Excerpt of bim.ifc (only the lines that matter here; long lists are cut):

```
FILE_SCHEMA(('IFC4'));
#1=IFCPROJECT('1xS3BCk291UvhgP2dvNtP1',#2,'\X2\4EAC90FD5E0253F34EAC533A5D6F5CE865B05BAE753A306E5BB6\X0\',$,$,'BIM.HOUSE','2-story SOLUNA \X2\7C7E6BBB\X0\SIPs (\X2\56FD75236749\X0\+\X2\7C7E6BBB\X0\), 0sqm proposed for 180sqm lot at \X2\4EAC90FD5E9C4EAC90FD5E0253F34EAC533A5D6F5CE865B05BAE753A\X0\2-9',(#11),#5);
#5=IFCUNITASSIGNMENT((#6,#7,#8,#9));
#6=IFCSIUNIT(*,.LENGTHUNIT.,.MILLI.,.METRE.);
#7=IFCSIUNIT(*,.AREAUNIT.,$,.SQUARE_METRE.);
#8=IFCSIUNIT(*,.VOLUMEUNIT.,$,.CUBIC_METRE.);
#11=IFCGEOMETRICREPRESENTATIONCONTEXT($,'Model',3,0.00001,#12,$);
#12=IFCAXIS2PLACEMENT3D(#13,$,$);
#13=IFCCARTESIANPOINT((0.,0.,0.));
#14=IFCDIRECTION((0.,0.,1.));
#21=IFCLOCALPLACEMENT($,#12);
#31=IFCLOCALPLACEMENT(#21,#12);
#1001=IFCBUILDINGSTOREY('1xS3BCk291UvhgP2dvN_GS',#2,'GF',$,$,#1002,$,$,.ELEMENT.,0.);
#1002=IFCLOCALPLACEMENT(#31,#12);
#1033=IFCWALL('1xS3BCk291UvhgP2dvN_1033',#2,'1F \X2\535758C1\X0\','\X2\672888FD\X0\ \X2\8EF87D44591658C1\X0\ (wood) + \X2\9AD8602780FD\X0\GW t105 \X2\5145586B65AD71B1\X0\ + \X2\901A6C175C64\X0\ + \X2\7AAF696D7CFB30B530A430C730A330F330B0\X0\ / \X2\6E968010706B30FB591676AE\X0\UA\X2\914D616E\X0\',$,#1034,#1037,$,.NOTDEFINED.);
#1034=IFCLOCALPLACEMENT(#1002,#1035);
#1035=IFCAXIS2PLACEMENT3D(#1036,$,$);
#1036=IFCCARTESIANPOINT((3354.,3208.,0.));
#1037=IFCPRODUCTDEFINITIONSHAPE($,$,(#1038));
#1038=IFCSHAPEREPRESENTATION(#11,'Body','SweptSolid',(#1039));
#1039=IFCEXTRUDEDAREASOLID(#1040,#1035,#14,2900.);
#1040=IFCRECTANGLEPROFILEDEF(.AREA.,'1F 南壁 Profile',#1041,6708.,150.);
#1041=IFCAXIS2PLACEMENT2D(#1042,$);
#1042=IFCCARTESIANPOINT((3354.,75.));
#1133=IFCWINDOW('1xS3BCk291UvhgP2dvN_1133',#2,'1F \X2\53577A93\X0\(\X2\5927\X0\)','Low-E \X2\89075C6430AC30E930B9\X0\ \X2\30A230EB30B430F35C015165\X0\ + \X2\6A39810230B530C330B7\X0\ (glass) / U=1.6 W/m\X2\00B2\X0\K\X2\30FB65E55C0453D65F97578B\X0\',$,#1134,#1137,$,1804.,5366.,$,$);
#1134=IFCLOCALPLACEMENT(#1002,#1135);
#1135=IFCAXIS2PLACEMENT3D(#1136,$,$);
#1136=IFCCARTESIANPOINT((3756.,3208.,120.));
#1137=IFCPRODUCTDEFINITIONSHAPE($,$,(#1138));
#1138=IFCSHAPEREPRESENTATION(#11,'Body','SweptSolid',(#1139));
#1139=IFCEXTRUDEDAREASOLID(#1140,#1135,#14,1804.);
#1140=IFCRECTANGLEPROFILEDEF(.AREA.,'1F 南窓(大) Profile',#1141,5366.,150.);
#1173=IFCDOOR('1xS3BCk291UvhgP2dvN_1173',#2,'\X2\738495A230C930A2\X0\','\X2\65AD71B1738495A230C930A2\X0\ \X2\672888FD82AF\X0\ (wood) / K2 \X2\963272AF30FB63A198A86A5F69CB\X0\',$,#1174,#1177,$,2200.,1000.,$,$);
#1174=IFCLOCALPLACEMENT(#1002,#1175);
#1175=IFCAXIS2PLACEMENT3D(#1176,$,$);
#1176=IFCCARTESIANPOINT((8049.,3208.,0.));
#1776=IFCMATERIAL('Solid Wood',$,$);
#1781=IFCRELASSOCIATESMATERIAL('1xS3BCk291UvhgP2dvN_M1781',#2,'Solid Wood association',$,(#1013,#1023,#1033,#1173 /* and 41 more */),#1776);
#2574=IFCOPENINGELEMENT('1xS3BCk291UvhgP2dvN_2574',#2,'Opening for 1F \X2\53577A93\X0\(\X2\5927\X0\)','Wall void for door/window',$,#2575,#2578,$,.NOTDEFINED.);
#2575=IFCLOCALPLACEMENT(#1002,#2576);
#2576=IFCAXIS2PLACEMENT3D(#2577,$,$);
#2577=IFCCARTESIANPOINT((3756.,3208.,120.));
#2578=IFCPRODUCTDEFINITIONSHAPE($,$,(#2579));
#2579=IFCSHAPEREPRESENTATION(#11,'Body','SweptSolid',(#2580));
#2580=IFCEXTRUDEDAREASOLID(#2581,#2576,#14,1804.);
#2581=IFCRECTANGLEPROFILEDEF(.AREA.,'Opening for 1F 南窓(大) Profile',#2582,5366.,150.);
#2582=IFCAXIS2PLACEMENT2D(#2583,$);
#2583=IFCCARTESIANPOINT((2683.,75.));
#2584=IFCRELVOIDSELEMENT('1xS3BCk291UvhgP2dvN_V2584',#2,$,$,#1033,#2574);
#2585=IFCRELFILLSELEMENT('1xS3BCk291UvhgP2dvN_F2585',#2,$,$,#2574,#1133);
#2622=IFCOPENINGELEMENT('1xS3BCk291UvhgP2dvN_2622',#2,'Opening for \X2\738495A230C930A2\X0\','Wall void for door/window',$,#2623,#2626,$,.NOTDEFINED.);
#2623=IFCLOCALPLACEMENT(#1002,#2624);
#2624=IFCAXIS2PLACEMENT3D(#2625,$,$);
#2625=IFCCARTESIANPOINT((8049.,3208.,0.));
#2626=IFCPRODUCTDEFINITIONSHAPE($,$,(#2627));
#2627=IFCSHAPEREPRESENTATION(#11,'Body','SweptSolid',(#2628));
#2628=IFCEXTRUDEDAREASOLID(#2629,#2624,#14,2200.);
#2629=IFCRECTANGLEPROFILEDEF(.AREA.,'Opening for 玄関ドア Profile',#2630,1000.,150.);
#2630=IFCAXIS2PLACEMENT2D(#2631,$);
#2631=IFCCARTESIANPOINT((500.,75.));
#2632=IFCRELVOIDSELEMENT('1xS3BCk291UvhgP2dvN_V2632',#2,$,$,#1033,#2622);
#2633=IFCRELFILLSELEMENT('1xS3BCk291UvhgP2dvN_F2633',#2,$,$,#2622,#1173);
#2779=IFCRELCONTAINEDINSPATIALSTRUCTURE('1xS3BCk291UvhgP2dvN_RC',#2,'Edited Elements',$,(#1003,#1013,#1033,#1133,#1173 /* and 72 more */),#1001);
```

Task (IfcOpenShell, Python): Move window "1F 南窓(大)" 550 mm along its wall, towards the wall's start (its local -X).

```python
import ifcopenshell
import ifcopenshell.api.geometry
import ifcopenshell.util.placement

model = ifcopenshell.open("bim.ifc")

window = model.by_guid("1xS3BCk291UvhgP2dvN_1133")
opening = window.FillsVoids[0].RelatingOpeningElement
wall = opening.VoidsElements[0].RelatingBuildingElement

wall_matrix = ifcopenshell.util.placement.get_local_placement(wall.ObjectPlacement)
shift = wall_matrix[:3, 0] * -550.0
before = ifcopenshell.util.placement.get_local_placement(window.ObjectPlacement)[:3, 3].copy()

# The window is not placed relative to its opening, so move both.
for product in (opening, window):
    matrix = ifcopenshell.util.placement.get_local_placement(product.ObjectPlacement)
    matrix[:3, 3] += shift
    ifcopenshell.api.geometry.edit_object_placement(model, product=product, matrix=matrix, is_si=False)

after = ifcopenshell.util.placement.get_local_placement(window.ObjectPlacement)[:3, 3]
print("window moved by", (after - before).round(3) + 0.0)

model.write("bim-out.ifc")
```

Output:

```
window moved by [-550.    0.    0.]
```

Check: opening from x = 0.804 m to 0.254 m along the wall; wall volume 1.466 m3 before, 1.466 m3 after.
